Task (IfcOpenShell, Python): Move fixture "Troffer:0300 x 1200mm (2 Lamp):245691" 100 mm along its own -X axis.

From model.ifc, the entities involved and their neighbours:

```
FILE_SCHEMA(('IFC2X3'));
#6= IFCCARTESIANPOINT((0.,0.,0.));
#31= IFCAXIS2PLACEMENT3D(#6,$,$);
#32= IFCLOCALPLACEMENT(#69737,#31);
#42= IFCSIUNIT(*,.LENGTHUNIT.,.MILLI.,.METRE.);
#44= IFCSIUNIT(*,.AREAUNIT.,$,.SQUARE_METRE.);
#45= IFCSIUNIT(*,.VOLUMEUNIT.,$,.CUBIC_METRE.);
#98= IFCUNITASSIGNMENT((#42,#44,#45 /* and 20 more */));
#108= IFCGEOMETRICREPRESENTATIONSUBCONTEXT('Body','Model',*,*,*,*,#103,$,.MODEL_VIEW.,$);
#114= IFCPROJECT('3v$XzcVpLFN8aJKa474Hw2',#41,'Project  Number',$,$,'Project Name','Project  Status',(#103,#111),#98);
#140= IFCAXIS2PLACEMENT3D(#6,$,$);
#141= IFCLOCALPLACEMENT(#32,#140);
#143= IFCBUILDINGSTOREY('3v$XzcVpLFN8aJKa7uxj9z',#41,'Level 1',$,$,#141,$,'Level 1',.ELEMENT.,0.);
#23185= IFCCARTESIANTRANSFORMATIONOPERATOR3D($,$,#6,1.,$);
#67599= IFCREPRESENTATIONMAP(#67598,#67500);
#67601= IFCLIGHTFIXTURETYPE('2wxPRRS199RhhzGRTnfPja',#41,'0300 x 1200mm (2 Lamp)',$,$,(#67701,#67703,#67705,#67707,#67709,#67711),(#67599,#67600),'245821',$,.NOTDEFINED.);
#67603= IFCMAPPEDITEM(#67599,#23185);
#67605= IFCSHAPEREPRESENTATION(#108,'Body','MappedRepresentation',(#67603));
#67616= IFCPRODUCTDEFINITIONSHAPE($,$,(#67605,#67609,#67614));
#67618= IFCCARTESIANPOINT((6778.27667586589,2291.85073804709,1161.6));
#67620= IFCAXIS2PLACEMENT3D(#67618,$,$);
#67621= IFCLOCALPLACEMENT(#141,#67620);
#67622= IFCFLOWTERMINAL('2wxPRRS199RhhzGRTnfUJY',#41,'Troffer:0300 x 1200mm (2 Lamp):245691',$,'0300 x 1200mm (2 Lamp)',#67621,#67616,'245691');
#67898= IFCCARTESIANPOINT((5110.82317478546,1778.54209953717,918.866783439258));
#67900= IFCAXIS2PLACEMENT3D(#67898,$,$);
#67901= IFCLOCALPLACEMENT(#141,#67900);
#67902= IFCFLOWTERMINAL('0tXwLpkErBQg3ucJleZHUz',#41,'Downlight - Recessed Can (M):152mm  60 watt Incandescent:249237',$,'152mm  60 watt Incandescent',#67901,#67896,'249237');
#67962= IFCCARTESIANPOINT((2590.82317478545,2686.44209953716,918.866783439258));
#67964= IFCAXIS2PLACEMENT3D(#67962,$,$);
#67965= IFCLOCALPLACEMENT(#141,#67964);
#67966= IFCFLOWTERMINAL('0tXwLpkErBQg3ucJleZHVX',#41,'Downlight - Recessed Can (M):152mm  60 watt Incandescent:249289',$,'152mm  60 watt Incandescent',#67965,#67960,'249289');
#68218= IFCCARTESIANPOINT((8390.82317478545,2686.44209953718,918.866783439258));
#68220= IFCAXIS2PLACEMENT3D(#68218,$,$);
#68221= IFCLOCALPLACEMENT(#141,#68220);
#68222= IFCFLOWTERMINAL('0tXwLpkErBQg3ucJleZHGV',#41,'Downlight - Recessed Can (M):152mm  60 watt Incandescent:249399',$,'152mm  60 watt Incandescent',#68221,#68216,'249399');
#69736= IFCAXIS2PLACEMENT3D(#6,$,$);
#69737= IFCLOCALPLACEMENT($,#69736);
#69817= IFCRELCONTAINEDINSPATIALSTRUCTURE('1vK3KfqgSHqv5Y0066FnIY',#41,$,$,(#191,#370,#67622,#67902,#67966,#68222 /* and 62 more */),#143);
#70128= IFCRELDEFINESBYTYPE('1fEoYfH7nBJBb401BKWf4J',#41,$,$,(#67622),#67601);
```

```python
import ifcopenshell
import ifcopenshell.api.geometry
import ifcopenshell.util.placement
import ifcopenshell.util.unit

model = ifcopenshell.open("model.ifc")
unit_scale = ifcopenshell.util.unit.calculate_unit_scale(model)

item = model.by_guid("2wxPRRS199RhhzGRTnfUJY")
matrix = ifcopenshell.util.placement.get_local_placement(item.ObjectPlacement)
matrix[:3, 3] -= matrix[:3, 0] * 0.1 / unit_scale
ifcopenshell.api.geometry.edit_object_placement(model, product=item, matrix=matrix, is_si=False)

print(ifcopenshell.util.placement.get_local_placement(item.ObjectPlacement).round(3) + 0.0)

model.write("model_updated.ifc")
```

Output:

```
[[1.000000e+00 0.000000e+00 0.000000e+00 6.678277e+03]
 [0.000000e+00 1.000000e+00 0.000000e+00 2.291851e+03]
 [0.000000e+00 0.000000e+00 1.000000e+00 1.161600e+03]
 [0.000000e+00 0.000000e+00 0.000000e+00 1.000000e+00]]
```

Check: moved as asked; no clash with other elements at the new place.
